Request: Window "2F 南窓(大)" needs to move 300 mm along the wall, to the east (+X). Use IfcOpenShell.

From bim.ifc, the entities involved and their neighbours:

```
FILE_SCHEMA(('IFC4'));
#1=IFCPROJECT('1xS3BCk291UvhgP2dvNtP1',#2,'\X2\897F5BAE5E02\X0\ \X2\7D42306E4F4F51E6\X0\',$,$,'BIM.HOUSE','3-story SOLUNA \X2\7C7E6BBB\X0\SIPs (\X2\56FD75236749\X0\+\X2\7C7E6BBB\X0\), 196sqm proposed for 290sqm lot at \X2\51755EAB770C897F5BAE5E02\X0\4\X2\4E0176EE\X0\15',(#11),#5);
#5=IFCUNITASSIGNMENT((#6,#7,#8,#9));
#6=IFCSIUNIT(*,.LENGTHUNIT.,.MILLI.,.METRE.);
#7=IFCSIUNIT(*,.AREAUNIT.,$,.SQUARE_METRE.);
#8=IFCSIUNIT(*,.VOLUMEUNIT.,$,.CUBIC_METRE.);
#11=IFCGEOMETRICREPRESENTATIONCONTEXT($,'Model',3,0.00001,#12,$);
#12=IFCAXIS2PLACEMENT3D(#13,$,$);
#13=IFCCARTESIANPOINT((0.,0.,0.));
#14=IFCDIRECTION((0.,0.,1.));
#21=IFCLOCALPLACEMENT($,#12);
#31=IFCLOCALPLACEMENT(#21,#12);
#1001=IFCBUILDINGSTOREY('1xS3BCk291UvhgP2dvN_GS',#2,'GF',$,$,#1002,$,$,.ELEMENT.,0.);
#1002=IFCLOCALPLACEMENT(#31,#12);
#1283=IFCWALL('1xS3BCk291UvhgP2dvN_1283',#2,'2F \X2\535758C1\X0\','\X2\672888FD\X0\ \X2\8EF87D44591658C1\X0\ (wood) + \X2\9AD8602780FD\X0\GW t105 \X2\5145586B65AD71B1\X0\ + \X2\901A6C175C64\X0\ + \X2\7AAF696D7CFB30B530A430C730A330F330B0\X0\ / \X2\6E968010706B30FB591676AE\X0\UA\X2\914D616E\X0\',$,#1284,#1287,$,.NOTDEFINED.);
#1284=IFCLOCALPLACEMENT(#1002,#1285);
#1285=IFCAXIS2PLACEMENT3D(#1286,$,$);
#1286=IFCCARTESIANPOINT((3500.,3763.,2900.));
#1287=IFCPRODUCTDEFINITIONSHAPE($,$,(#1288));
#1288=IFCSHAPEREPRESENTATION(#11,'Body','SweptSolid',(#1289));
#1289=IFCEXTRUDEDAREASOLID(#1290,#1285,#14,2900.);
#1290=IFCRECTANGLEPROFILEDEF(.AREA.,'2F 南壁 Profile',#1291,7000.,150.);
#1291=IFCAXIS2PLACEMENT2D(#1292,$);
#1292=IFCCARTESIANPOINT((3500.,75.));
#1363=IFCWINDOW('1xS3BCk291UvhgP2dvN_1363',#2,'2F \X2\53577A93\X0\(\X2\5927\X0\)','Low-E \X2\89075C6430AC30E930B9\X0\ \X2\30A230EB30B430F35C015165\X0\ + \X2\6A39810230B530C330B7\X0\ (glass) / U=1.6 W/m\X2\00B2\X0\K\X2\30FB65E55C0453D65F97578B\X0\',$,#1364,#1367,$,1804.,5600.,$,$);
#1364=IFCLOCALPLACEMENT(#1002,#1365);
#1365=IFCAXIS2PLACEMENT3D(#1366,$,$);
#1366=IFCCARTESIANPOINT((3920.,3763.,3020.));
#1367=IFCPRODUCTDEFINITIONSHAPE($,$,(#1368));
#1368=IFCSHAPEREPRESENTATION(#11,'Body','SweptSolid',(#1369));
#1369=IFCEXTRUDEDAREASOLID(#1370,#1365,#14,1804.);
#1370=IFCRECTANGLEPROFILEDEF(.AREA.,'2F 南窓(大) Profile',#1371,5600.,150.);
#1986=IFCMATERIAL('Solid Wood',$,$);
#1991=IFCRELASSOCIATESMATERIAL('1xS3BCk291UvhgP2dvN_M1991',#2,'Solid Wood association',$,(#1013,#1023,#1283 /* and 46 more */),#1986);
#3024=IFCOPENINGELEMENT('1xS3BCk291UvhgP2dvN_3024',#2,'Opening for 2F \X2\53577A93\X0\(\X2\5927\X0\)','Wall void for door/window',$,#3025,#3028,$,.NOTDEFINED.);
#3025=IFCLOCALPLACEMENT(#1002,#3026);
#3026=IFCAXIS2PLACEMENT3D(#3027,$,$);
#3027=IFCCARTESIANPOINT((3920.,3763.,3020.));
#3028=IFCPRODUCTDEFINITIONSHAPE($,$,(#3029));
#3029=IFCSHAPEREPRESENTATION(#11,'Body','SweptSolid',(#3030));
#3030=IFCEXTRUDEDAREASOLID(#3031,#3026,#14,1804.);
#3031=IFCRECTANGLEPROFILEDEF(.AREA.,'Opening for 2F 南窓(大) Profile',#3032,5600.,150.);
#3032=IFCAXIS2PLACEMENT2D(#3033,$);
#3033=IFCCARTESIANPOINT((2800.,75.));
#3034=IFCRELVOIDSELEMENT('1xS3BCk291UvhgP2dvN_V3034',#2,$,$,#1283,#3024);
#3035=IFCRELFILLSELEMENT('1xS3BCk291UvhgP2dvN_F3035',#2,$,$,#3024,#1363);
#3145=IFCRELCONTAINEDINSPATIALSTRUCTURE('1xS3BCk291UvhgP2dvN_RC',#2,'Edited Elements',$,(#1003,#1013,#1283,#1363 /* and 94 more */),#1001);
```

```python
import ifcopenshell
import ifcopenshell.api.geometry
import ifcopenshell.util.placement

model = ifcopenshell.open("bim.ifc")

window = model.by_guid("1xS3BCk291UvhgP2dvN_1363")
opening = window.FillsVoids[0].RelatingOpeningElement
wall = opening.VoidsElements[0].RelatingBuildingElement

wall_matrix = ifcopenshell.util.placement.get_local_placement(wall.ObjectPlacement)
shift = wall_matrix[:3, 0] * 300.0
before = ifcopenshell.util.placement.get_local_placement(window.ObjectPlacement)[:3, 3].copy()

# The window is not placed relative to its opening, so move both.
for product in (opening, window):
    matrix = ifcopenshell.util.placement.get_local_placement(product.ObjectPlacement)
    matrix[:3, 3] += shift
    ifcopenshell.api.geometry.edit_object_placement(model, product=product, matrix=matrix, is_si=False)

after = ifcopenshell.util.placement.get_local_placement(window.ObjectPlacement)[:3, 3]
print("window moved by", (after - before).round(3) + 0.0)

model.write("bim_edited.ifc")
```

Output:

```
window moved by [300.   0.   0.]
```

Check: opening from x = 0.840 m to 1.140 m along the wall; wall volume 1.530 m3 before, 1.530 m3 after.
